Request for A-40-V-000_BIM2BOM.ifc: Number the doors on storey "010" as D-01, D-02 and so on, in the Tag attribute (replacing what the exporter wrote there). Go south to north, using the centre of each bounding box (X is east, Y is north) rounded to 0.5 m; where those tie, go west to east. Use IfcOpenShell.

First a look at what the model holds.

```python
import ifcopenshell
import ifcopenshell.util.element
import ifcopenshell.util.placement

model = ifcopenshell.open("A-40-V-000_BIM2BOM.ifc")
print(model.schema)
storey = next(s for s in model.by_type("IfcBuildingStorey") if s.Name == "010")
doors = [e for e in ifcopenshell.util.element.get_decomposition(storey) if e.is_a("IfcDoor")]
for e in sorted(doors, key=lambda e: e.id()):
    origin = ifcopenshell.util.placement.get_local_placement(e.ObjectPlacement)[:3, 3]
    print(e.id(), e.Tag, e.Name, origin.round(2) + 0.0, sep=" | ")
```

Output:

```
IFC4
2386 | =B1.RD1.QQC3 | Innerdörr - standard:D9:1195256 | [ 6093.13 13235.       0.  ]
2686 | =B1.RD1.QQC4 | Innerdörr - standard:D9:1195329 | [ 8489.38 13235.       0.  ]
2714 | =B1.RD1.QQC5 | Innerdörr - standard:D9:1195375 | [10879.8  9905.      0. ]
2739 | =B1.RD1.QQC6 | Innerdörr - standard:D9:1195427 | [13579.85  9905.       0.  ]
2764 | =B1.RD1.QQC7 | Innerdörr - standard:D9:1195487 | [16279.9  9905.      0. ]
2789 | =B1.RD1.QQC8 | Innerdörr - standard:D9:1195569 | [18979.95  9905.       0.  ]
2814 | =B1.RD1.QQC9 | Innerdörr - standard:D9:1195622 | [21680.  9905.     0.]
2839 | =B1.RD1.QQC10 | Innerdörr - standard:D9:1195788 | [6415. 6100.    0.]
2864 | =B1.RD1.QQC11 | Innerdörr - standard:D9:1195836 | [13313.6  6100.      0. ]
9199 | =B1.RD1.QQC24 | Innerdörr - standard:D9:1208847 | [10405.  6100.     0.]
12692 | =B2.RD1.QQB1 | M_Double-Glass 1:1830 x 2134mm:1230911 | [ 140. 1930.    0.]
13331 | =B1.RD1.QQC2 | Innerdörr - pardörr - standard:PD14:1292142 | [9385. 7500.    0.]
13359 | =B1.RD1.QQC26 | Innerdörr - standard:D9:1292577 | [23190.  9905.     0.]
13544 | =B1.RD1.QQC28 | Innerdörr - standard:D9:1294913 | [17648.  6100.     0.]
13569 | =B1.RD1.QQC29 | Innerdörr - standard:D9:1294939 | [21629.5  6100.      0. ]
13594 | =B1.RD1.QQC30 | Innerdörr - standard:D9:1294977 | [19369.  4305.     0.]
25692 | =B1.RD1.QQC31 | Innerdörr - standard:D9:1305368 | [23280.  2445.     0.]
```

```python
import ifcopenshell
import ifcopenshell.geom
import ifcopenshell.util.element
import ifcopenshell.util.shape

model = ifcopenshell.open("A-40-V-000_BIM2BOM.ifc")
settings = ifcopenshell.geom.settings()
settings.set("use-world-coords", True)


def centre(element):
    shape = ifcopenshell.geom.create_shape(settings, element)
    return ifcopenshell.util.shape.get_bbox_centroid(shape.geometry)


storey = next(s for s in model.by_type("IfcBuildingStorey") if s.Name == "010")
doors = [e for e in ifcopenshell.util.element.get_decomposition(storey) if e.is_a("IfcDoor")]

# Insertion points can sit at a corner or the storey origin, so sort by the geometry (in metres).
centres = {e: centre(e) for e in doors}
doors.sort(key=lambda e: (round(centres[e][1] / 0.5), centres[e][0]))

for i, e in enumerate(doors, start=1):
    number = f"D-{i:02d}"
    e.Tag = number
    print(e.id(), number)

model.write("A-40-V-000_BIM2BOM_updated.ifc")
```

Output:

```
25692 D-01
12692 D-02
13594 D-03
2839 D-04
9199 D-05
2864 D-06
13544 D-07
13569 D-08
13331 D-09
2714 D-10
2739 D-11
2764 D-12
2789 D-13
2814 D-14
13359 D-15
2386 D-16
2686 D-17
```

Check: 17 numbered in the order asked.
